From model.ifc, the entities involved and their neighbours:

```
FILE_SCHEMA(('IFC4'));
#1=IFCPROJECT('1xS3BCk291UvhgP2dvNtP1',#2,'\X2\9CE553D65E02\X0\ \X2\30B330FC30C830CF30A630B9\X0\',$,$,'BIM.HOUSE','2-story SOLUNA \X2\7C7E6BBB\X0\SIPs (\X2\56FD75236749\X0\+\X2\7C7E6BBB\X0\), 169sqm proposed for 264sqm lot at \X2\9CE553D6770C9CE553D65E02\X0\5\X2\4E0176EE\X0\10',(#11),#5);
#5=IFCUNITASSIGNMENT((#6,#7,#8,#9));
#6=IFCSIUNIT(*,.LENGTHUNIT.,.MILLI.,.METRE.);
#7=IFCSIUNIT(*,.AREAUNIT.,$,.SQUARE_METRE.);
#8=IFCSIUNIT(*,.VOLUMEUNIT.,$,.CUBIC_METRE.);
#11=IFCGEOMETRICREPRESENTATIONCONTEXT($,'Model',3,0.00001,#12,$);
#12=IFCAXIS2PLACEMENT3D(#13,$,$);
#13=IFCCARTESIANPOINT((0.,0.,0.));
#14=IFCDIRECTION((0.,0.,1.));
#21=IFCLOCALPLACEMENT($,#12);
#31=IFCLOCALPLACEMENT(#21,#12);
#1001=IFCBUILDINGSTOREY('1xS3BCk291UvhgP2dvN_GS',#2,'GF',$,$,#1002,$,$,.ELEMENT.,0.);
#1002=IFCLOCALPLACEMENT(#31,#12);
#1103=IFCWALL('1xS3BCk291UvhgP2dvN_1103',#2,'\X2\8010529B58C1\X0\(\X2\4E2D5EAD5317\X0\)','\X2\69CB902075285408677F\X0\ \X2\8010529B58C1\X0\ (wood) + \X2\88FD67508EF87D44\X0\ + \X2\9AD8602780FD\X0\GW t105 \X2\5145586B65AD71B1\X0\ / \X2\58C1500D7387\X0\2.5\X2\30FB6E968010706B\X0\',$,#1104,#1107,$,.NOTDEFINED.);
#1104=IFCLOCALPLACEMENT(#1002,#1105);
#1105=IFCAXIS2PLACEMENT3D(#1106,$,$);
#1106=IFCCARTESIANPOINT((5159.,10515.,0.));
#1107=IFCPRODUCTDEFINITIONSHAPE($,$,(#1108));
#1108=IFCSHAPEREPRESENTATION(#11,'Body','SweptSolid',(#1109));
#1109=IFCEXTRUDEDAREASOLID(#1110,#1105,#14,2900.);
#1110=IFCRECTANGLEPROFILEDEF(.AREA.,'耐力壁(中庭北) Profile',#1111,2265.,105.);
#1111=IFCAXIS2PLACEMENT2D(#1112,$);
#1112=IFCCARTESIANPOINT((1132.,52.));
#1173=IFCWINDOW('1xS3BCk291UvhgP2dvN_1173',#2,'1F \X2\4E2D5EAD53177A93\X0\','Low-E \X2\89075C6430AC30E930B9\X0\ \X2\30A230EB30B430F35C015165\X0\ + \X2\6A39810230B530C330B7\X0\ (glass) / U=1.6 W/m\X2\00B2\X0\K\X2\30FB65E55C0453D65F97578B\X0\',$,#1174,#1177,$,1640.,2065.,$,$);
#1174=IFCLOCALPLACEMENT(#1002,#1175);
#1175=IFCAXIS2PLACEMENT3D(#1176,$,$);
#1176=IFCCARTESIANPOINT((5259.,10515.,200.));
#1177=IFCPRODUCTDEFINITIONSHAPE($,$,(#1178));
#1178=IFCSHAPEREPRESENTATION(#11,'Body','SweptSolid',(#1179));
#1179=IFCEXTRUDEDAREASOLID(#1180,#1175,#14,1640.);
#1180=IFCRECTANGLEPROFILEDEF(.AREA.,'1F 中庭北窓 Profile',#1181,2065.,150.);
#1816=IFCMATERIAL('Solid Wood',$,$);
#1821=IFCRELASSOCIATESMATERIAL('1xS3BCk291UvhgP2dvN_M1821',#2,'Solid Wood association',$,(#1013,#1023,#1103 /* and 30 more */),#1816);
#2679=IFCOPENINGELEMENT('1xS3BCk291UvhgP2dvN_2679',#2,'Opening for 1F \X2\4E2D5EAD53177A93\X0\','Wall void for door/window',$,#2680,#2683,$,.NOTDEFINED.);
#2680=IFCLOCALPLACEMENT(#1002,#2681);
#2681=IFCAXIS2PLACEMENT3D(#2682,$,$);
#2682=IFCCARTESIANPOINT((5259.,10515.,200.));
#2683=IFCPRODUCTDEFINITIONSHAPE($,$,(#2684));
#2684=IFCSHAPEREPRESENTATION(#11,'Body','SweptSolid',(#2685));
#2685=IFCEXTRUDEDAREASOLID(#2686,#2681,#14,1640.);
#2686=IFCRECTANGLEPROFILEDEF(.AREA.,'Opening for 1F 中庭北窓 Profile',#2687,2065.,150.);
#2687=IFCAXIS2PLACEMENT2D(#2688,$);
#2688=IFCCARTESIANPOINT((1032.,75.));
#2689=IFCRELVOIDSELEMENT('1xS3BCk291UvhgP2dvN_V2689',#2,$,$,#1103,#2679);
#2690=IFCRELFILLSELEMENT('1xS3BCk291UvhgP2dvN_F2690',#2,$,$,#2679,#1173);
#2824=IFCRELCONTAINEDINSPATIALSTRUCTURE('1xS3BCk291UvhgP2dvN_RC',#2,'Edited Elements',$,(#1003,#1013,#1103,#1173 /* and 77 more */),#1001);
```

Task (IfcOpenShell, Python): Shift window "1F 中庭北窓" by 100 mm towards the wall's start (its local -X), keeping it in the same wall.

```python
import ifcopenshell
import ifcopenshell.api.geometry
import ifcopenshell.util.placement
import ifcopenshell.util.unit

model = ifcopenshell.open("model.ifc")
unit_scale = ifcopenshell.util.unit.calculate_unit_scale(model)

window = model.by_guid("1xS3BCk291UvhgP2dvN_1173")
opening = window.FillsVoids[0].RelatingOpeningElement
wall = opening.VoidsElements[0].RelatingBuildingElement

wall_matrix = ifcopenshell.util.placement.get_local_placement(wall.ObjectPlacement)
shift = wall_matrix[:3, 0] * -0.1 / unit_scale
before = ifcopenshell.util.placement.get_local_placement(window.ObjectPlacement)[:3, 3].copy()

# The window is not placed relative to its opening, so move both.
for product in (opening, window):
    matrix = ifcopenshell.util.placement.get_local_placement(product.ObjectPlacement)
    matrix[:3, 3] += shift
    ifcopenshell.api.geometry.edit_object_placement(model, product=product, matrix=matrix, is_si=False)

after = ifcopenshell.util.placement.get_local_placement(window.ObjectPlacement)[:3, 3]
print("window moved by", (after - before).round(3) + 0.0)

model.write("model-out.ifc")
```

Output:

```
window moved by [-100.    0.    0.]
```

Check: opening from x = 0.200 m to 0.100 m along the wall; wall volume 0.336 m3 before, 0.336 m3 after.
